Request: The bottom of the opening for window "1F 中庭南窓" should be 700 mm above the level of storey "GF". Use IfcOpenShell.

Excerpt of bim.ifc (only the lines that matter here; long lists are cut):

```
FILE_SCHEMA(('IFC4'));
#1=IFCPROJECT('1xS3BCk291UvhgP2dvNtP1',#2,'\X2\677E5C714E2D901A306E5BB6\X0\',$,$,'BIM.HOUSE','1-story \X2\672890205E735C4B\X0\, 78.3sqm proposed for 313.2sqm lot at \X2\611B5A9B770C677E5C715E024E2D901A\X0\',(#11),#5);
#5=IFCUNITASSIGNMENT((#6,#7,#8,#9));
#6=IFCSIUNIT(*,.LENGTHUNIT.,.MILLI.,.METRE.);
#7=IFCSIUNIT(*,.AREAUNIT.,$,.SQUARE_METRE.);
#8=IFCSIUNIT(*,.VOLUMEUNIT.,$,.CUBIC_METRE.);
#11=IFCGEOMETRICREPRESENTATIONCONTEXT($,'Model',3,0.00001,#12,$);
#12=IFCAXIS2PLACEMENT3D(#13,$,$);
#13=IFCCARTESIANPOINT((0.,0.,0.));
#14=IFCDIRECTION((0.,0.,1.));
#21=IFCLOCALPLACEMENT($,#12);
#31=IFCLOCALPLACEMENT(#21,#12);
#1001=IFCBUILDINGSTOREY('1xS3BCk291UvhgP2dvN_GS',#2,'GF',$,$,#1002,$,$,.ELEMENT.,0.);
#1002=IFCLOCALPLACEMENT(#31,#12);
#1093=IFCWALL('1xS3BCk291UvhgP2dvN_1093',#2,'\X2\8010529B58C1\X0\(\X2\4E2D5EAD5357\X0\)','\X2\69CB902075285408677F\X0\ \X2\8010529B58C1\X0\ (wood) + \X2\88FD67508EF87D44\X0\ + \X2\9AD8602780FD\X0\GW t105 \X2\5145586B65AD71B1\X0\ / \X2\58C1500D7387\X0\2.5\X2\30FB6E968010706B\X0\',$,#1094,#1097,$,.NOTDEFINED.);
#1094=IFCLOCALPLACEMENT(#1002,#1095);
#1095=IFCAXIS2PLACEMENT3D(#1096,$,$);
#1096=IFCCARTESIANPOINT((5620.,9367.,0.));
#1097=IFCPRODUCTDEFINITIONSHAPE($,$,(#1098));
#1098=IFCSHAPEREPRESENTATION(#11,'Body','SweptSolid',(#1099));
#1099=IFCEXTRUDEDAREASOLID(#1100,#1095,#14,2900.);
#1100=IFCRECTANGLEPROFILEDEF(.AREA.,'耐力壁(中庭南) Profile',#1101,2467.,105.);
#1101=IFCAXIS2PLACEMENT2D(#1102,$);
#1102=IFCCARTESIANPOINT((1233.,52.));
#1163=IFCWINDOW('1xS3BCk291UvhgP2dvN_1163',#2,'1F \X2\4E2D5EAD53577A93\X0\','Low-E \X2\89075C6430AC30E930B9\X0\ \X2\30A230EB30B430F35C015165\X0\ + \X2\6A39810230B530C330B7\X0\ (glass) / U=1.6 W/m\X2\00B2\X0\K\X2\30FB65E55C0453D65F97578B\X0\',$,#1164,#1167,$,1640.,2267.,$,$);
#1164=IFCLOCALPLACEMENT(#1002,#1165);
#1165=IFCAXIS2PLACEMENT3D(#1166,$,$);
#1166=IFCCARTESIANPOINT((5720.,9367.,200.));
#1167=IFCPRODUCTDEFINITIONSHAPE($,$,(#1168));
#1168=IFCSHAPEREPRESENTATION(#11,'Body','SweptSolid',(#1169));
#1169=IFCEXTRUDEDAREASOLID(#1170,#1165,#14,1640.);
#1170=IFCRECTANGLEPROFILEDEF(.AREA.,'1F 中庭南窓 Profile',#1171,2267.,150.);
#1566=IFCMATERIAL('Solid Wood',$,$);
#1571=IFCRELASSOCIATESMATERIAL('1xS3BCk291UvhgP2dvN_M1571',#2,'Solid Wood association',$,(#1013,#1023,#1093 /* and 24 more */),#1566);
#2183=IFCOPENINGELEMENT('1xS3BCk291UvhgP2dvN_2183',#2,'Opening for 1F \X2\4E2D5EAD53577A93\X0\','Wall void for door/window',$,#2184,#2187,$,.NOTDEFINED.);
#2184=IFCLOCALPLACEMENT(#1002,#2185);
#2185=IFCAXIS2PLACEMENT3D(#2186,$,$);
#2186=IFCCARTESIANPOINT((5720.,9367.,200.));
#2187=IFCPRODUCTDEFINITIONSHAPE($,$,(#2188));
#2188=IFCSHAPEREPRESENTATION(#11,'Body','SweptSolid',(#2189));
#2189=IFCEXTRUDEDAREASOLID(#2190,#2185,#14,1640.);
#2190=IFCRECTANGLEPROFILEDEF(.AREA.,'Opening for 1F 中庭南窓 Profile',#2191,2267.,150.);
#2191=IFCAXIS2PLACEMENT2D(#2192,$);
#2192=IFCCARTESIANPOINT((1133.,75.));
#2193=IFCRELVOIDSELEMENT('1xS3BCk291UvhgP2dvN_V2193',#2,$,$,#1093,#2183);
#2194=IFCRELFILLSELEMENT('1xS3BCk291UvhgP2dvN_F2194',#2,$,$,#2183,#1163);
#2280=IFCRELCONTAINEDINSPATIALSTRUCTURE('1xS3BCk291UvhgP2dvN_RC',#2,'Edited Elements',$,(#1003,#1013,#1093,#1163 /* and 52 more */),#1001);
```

```python
import numpy as np
import ifcopenshell
import ifcopenshell.api.geometry
import ifcopenshell.geom
import ifcopenshell.util.element
import ifcopenshell.util.placement
import ifcopenshell.util.shape
import ifcopenshell.util.unit

model = ifcopenshell.open("bim.ifc")
unit_scale = ifcopenshell.util.unit.calculate_unit_scale(model)

window = model.by_id(1163)
opening = window.FillsVoids[0].RelatingOpeningElement
storey = ifcopenshell.util.element.get_container(window, ifc_class="IfcBuildingStorey")
level = ifcopenshell.util.placement.get_local_placement(storey.ObjectPlacement)[2, 3]

# The opening's origin need not be at the sill, so measure its lowest point.
shape = ifcopenshell.geom.create_shape(ifcopenshell.geom.settings(), opening)
bottom = ifcopenshell.util.shape.get_shape_bottom_elevation(shape, shape.geometry) / unit_scale
dz = level + 700.0 - bottom

shift = np.array([0.0, 0.0, dz])
# The window is not placed relative to its opening, so move both.
for product in (opening, window):
    matrix = ifcopenshell.util.placement.get_local_placement(product.ObjectPlacement)
    matrix[:3, 3] += shift
    ifcopenshell.api.geometry.edit_object_placement(model, product=product, matrix=matrix, is_si=False)

print(f"moved by {dz * unit_scale:+.3f} m")

model.write("bim-out.ifc")
```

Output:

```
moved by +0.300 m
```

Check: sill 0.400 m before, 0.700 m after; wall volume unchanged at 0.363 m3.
